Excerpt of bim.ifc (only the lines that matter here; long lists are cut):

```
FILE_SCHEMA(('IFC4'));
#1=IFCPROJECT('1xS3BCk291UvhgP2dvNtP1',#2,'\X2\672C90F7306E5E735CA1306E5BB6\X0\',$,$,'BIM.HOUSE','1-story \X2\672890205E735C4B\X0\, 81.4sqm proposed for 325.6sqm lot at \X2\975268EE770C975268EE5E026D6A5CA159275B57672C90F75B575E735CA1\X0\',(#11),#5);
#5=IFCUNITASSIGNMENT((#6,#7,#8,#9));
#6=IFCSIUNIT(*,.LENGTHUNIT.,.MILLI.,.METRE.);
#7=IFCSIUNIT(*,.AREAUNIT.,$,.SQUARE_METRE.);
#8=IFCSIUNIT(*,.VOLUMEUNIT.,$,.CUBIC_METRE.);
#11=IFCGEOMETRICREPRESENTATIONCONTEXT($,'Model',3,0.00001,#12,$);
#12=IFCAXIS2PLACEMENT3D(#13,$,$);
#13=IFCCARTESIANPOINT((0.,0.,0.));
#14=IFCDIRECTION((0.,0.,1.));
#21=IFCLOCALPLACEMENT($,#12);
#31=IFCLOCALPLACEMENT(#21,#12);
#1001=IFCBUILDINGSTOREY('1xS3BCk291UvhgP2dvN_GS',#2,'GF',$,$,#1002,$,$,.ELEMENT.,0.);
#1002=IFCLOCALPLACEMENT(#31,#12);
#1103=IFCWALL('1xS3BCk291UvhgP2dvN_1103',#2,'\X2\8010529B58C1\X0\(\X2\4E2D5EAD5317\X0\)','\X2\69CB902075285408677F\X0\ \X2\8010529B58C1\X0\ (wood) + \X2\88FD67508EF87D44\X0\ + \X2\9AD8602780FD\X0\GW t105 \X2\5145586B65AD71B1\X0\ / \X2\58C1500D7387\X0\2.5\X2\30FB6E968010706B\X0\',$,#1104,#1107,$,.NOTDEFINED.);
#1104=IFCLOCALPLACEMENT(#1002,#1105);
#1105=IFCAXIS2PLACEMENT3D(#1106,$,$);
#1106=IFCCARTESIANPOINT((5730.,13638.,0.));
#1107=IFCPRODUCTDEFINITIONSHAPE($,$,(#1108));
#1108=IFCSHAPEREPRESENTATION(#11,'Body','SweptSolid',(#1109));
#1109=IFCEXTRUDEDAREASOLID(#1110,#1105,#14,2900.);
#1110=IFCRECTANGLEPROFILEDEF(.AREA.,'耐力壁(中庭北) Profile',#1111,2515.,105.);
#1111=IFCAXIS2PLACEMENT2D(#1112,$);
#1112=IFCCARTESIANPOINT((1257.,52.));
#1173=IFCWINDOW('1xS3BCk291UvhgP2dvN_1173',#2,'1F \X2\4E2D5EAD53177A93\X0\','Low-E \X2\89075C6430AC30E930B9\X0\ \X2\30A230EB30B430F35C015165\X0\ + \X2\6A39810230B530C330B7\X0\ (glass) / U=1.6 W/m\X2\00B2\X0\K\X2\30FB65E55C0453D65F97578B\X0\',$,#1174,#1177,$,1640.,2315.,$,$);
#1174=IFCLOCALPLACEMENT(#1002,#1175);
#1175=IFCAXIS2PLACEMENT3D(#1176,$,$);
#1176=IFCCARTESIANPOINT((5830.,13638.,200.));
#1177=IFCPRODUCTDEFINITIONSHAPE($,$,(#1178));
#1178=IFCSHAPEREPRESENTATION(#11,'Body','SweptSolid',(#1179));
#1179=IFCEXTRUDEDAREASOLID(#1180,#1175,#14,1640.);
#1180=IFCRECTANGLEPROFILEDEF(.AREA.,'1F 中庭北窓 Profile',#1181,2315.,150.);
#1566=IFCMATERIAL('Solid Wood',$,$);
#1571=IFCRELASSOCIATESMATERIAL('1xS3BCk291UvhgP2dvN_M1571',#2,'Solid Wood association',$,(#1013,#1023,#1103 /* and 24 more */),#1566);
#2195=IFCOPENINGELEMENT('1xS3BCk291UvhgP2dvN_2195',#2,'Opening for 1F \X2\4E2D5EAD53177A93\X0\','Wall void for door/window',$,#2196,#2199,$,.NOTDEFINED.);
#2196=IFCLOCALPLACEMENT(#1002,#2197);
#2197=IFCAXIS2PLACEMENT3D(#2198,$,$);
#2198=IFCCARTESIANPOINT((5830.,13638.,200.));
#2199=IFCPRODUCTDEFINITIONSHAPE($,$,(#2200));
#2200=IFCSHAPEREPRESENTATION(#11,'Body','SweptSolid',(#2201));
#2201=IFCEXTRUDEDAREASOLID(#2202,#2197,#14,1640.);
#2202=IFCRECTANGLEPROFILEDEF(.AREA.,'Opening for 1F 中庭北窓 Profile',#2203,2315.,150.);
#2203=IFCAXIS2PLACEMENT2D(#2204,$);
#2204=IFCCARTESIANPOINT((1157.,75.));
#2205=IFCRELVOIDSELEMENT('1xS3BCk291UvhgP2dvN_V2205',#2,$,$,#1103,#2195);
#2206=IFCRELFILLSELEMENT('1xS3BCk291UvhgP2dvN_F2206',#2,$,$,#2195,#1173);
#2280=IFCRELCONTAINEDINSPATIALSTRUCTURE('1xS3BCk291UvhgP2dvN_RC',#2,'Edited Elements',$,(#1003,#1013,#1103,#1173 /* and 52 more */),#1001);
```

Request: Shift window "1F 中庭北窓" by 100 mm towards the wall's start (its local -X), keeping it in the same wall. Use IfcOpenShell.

```python
import ifcopenshell
import ifcopenshell.api.geometry
import ifcopenshell.util.placement
import ifcopenshell.util.unit

model = ifcopenshell.open("bim.ifc")
unit_scale = ifcopenshell.util.unit.calculate_unit_scale(model)

window = model.by_guid("1xS3BCk291UvhgP2dvN_1173")
opening = window.FillsVoids[0].RelatingOpeningElement
wall = opening.VoidsElements[0].RelatingBuildingElement

wall_matrix = ifcopenshell.util.placement.get_local_placement(wall.ObjectPlacement)
shift = wall_matrix[:3, 0] * -0.1 / unit_scale
before = ifcopenshell.util.placement.get_local_placement(window.ObjectPlacement)[:3, 3].copy()

# The window is not placed relative to its opening, so move both.
for product in (opening, window):
    matrix = ifcopenshell.util.placement.get_local_placement(product.ObjectPlacement)
    matrix[:3, 3] += shift
    ifcopenshell.api.geometry.edit_object_placement(model, product=product, matrix=matrix, is_si=False)

after = ifcopenshell.util.placement.get_local_placement(window.ObjectPlacement)[:3, 3]
print("window moved by", (after - before).round(3) + 0.0)

model.write("bim-out.ifc")
```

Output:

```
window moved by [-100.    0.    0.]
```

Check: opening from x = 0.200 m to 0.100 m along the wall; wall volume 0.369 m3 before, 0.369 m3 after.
